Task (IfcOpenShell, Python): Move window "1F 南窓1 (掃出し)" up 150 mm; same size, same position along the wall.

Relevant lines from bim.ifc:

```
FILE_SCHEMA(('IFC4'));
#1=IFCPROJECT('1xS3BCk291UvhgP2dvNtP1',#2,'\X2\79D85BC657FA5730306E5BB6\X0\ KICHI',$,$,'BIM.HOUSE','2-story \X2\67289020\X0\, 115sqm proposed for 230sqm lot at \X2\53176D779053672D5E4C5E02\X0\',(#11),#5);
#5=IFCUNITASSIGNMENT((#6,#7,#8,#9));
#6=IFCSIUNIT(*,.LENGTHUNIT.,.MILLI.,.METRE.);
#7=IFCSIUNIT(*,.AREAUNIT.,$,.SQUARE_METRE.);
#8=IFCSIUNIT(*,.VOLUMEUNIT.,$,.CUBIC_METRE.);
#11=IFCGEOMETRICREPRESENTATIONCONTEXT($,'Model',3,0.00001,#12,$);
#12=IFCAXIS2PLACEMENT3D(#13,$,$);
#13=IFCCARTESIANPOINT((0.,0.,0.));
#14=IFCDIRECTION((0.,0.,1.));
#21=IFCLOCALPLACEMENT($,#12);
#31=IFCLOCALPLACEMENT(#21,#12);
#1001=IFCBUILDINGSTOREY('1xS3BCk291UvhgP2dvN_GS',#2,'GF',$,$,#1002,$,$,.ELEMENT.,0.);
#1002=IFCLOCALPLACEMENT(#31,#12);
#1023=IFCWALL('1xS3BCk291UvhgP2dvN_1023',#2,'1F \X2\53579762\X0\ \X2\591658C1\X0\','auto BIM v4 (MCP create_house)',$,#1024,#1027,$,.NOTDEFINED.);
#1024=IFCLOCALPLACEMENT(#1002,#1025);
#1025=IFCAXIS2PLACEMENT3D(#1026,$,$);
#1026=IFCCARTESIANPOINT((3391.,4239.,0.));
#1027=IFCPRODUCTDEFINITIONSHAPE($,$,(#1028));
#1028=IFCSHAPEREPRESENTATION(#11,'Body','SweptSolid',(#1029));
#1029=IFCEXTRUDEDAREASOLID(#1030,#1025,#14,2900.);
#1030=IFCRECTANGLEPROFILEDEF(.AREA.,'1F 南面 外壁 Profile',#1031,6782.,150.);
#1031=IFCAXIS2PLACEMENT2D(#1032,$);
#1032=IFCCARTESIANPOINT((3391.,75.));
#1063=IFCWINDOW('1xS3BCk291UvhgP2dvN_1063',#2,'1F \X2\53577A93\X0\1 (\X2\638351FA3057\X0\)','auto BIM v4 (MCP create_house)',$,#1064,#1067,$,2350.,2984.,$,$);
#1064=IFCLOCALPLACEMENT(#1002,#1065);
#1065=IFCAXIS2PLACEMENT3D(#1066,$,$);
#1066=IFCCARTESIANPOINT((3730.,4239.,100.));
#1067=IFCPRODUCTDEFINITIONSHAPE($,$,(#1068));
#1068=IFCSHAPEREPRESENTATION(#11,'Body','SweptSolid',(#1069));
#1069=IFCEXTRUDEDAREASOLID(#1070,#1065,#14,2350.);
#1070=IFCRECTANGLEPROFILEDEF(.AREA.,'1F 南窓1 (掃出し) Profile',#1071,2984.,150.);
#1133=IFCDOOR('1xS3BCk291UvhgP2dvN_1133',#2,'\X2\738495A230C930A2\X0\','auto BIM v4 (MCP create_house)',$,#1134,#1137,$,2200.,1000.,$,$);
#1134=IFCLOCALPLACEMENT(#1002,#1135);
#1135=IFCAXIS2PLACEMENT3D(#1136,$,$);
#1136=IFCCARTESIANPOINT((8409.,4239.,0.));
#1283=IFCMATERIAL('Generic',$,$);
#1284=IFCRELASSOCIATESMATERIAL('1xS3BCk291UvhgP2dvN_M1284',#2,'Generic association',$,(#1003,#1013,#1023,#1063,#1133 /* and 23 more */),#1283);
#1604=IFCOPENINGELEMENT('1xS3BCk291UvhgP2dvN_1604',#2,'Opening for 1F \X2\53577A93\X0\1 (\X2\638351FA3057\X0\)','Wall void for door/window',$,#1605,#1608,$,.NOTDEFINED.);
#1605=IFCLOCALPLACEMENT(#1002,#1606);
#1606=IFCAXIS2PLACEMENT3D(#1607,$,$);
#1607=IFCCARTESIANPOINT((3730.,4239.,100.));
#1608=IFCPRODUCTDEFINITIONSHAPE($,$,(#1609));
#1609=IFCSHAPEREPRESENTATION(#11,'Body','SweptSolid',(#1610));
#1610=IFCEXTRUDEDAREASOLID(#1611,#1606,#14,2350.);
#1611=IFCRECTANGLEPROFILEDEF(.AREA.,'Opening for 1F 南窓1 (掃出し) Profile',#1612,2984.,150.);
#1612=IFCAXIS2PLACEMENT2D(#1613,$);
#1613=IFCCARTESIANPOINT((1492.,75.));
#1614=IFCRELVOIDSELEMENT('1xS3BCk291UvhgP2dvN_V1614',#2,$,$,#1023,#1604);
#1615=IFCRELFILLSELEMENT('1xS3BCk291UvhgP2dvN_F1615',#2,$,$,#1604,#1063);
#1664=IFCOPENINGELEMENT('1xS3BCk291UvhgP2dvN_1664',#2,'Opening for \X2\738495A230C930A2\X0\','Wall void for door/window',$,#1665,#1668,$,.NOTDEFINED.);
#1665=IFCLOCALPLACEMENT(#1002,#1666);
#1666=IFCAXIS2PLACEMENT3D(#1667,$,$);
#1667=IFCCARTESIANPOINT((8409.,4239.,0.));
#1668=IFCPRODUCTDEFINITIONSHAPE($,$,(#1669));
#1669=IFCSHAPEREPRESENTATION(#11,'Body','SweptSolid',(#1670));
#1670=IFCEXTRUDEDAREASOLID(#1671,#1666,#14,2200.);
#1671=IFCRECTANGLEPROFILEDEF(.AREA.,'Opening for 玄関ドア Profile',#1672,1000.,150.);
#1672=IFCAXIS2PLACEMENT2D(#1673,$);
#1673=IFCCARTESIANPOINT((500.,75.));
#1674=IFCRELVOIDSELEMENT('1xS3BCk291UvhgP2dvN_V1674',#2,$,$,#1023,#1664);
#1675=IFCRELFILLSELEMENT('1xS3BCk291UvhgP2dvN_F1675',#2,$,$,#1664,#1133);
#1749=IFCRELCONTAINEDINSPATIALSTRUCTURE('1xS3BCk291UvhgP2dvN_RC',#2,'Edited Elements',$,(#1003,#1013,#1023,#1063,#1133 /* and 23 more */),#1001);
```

```python
import numpy as np
import ifcopenshell
import ifcopenshell.api.geometry
import ifcopenshell.util.placement
import ifcopenshell.util.unit

model = ifcopenshell.open("bim.ifc")
unit_scale = ifcopenshell.util.unit.calculate_unit_scale(model)

window = model.by_guid("1xS3BCk291UvhgP2dvN_1063")
opening = window.FillsVoids[0].RelatingOpeningElement
dz = 0.15 / unit_scale

shift = np.array([0.0, 0.0, dz])
# The window is not placed relative to its opening, so move both.
for product in (opening, window):
    matrix = ifcopenshell.util.placement.get_local_placement(product.ObjectPlacement)
    matrix[:3, 3] += shift
    ifcopenshell.api.geometry.edit_object_placement(model, product=product, matrix=matrix, is_si=False)

print(f"moved by {dz * unit_scale:+.3f} m")

model.write("bim_updated.ifc")
```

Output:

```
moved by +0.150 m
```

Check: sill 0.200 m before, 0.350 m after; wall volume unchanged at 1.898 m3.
